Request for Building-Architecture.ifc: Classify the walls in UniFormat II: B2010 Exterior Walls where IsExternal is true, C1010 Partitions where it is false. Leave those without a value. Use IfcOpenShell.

First a look at what the model holds.

```python
import ifcopenshell
import ifcopenshell.util.element

model = ifcopenshell.open("Building-Architecture.ifc")
print(model.schema)
print("classifications:", [c.Name for c in model.by_type("IfcClassification")])
values = [ifcopenshell.util.element.get_pset(e, "Pset_WallCommon", "IsExternal") for e in model.by_type("IfcWall")]
for value in (True, False, None):
    print("IsExternal", value, values.count(value))
```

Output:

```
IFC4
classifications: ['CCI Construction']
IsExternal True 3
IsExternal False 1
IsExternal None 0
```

```python
import ifcopenshell
import ifcopenshell.api.classification
import ifcopenshell.util.element

model = ifcopenshell.open("Building-Architecture.ifc")

system = ifcopenshell.api.classification.add_classification(model, classification="UniFormat II")

walls = model.by_type("IfcWall")
external = {e: ifcopenshell.util.element.get_pset(e, "Pset_WallCommon", "IsExternal") for e in walls}
for flag, code, name in ((True, "B2010", "Exterior Walls"), (False, "C1010", "Partitions")):
    products = [e for e in walls if external[e] is flag]
    ifcopenshell.api.classification.add_reference(
        model, products=products, classification=system, identification=code, name=name
    )
    print(code, len(products))

model.write("Building-Architecture_v2.ifc")
```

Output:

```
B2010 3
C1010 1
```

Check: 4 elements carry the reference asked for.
